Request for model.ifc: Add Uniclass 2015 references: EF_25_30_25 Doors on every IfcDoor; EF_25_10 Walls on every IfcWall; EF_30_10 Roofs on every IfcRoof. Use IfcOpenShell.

First a look at what the model holds.

```python
import ifcopenshell

model = ifcopenshell.open("model.ifc")
print(model.schema)
print("classifications:", [c.Name for c in model.by_type("IfcClassification")])
for ifc_class in ("IfcDoor", "IfcRoof", "IfcStair", "IfcWall", "IfcWindow"):
    print(ifc_class, len(model.by_type(ifc_class)))
```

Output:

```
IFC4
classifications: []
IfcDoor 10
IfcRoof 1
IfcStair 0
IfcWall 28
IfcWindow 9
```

```python
import ifcopenshell
import ifcopenshell.api.classification

model = ifcopenshell.open("model.ifc")

system = ifcopenshell.api.classification.add_classification(model, classification="Uniclass 2015")

codes = {
    "IfcDoor": ("EF_25_30_25", "Doors"),
    "IfcWall": ("EF_25_10", "Walls"),
    "IfcRoof": ("EF_30_10", "Roofs"),
}
for ifc_class, (code, name) in codes.items():
    products = model.by_type(ifc_class)
    ifcopenshell.api.classification.add_reference(
        model, products=products, classification=system, identification=code, name=name
    )
    print(code, len(products))

model.write("model_edited.ifc")
```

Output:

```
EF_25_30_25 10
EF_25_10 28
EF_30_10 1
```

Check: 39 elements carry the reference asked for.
